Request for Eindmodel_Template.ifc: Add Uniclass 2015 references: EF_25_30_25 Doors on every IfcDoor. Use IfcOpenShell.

First a look at what the model holds.

```python
import ifcopenshell

model = ifcopenshell.open("Eindmodel_Template.ifc")
print(model.schema)
print("classifications:", [c.Name for c in model.by_type("IfcClassification")])
for ifc_class in ("IfcDoor", "IfcRoof", "IfcStair", "IfcWall", "IfcWindow"):
    print(ifc_class, len(model.by_type(ifc_class)))
```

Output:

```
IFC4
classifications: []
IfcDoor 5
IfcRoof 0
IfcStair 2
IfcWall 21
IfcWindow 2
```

```python
import ifcopenshell
import ifcopenshell.api.classification

model = ifcopenshell.open("Eindmodel_Template.ifc")

system = ifcopenshell.api.classification.add_classification(model, classification="Uniclass 2015")

codes = {
    "IfcDoor": ("EF_25_30_25", "Doors"),
}
for ifc_class, (code, name) in codes.items():
    products = model.by_type(ifc_class)
    ifcopenshell.api.classification.add_reference(
        model, products=products, classification=system, identification=code, name=name
    )
    print(code, len(products))

model.write("Eindmodel_Template_updated.ifc")
```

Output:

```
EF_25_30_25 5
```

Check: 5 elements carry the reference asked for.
